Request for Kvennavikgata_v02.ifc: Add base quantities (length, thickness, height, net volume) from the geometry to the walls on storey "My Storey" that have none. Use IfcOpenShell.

First a look at what the model holds.

```python
import ifcopenshell
import ifcopenshell.util.element
import ifcopenshell.util.unit

model = ifcopenshell.open("Kvennavikgata_v02.ifc")
print(model.schema)
for unit_type in ("LENGTHUNIT", "AREAUNIT", "VOLUMEUNIT"):
    print(unit_type, ifcopenshell.util.unit.calculate_unit_scale(model, unit_type))
storey = next(s for s in model.by_type("IfcBuildingStorey") if s.Name == "My Storey")
walls = [e for e in ifcopenshell.util.element.get_decomposition(storey) if e.is_a("IfcWall")]
for e in sorted(walls, key=lambda e: e.id()):
    print(e.id(), e.is_a(), e.Name, list(ifcopenshell.util.element.get_psets(e, qtos_only=True)), sep=" | ")
```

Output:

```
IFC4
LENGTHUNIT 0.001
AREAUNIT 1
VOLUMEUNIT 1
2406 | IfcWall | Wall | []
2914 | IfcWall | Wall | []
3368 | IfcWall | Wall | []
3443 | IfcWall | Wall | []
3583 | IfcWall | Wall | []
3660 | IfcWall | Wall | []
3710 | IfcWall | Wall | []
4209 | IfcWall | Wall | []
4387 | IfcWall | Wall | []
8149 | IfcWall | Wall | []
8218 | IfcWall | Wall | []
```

```python
import ifcopenshell
import ifcopenshell.api.pset
import ifcopenshell.geom
import ifcopenshell.util.element
import ifcopenshell.util.shape
import ifcopenshell.util.unit

model = ifcopenshell.open("Kvennavikgata_v02.ifc")
unit_scale = ifcopenshell.util.unit.calculate_unit_scale(model)
volume_scale = ifcopenshell.util.unit.calculate_unit_scale(model, "VOLUMEUNIT")
settings = ifcopenshell.geom.settings()

storey = next(s for s in model.by_type("IfcBuildingStorey") if s.Name == "My Storey")
walls = [e for e in ifcopenshell.util.element.get_decomposition(storey) if e.is_a("IfcWall")]

for e in sorted(walls, key=lambda e: e.id()):
    if ifcopenshell.util.element.get_psets(e, qtos_only=True, should_inherit=False):
        continue
    # Geometry comes back in metres, in the element's own axes.
    shape = ifcopenshell.geom.create_shape(settings, e)
    values = {
        "Length": ifcopenshell.util.shape.get_x(shape.geometry) / unit_scale,
        "Width": ifcopenshell.util.shape.get_y(shape.geometry) / unit_scale,
        "Height": ifcopenshell.util.shape.get_z(shape.geometry) / unit_scale,
        "NetVolume": ifcopenshell.util.shape.get_volume(shape.geometry) / volume_scale,
    }
    qto = ifcopenshell.api.pset.add_qto(model, product=e, name="Qto_WallBaseQuantities")
    ifcopenshell.api.pset.edit_qto(model, qto=qto, properties=values)
    print(e.id(), {k: round(v, 3) for k, v in values.items()})

model.write("Kvennavikgata_v02-out.ifc")
```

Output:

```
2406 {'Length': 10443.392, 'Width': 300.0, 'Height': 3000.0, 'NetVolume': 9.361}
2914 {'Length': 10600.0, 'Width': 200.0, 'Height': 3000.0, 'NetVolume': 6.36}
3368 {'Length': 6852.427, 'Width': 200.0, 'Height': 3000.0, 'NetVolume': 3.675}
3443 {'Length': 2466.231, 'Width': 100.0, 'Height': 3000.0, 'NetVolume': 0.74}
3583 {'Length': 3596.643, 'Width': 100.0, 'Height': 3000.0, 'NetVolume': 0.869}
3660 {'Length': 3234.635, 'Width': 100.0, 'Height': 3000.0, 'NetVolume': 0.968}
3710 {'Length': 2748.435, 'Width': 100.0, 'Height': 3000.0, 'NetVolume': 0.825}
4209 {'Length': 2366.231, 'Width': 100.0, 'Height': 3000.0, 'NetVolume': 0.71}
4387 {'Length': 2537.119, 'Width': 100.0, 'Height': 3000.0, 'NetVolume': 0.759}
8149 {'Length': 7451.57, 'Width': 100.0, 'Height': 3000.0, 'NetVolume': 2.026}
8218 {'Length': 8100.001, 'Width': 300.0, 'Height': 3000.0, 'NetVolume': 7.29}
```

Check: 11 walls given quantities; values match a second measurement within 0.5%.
